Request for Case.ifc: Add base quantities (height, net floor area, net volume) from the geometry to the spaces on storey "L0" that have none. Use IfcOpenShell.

First a look at what the model holds.

```python
import ifcopenshell
import ifcopenshell.util.element
import ifcopenshell.util.unit

model = ifcopenshell.open("Case.ifc")
print(model.schema)
for unit_type in ("LENGTHUNIT", "AREAUNIT", "VOLUMEUNIT"):
    print(unit_type, ifcopenshell.util.unit.calculate_unit_scale(model, unit_type))
storey = next(s for s in model.by_type("IfcBuildingStorey") if s.Name == "L0")
spaces = [e for e in ifcopenshell.util.element.get_decomposition(storey) if e.is_a("IfcSpace")]
for e in sorted(spaces, key=lambda e: e.id()):
    print(e.id(), e.is_a(), e.Name, list(ifcopenshell.util.element.get_psets(e, qtos_only=True)), sep=" | ")
```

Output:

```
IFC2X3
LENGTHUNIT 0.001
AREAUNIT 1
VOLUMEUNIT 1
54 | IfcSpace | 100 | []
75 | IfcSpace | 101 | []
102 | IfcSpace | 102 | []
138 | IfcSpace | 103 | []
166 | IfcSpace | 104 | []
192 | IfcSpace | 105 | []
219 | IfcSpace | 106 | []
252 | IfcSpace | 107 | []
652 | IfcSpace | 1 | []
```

```python
import ifcopenshell
import ifcopenshell.api.pset
import ifcopenshell.geom
import ifcopenshell.util.element
import ifcopenshell.util.shape
import ifcopenshell.util.unit

model = ifcopenshell.open("Case.ifc")
unit_scale = ifcopenshell.util.unit.calculate_unit_scale(model)
area_scale = ifcopenshell.util.unit.calculate_unit_scale(model, "AREAUNIT")
volume_scale = ifcopenshell.util.unit.calculate_unit_scale(model, "VOLUMEUNIT")
settings = ifcopenshell.geom.settings()

storey = next(s for s in model.by_type("IfcBuildingStorey") if s.Name == "L0")
spaces = [e for e in ifcopenshell.util.element.get_decomposition(storey) if e.is_a("IfcSpace")]

for e in sorted(spaces, key=lambda e: e.id()):
    if ifcopenshell.util.element.get_psets(e, qtos_only=True, should_inherit=False):
        continue
    # Geometry comes back in metres, in the element's own axes.
    shape = ifcopenshell.geom.create_shape(settings, e)
    values = {
        "Height": ifcopenshell.util.shape.get_z(shape.geometry) / unit_scale,
        "NetFloorArea": ifcopenshell.util.shape.get_footprint_area(shape.geometry) / area_scale,
        "NetVolume": ifcopenshell.util.shape.get_volume(shape.geometry) / volume_scale,
    }
    qto = ifcopenshell.api.pset.add_qto(model, product=e, name="BaseQuantities")
    ifcopenshell.api.pset.edit_qto(model, qto=qto, properties=values)
    print(e.id(), {k: round(v, 3) for k, v in values.items()})

model.write("Case_v2.ifc")
```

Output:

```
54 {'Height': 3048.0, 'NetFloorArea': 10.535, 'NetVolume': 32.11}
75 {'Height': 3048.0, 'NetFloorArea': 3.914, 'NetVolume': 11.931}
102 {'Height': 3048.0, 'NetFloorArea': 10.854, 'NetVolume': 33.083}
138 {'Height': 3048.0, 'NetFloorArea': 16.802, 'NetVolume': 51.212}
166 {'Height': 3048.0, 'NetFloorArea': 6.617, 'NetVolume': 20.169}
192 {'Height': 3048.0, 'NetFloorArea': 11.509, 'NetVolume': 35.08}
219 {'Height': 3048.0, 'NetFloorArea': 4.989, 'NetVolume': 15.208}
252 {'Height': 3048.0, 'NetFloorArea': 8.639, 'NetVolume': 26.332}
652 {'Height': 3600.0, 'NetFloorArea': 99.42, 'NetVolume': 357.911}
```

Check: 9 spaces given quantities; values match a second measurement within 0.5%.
